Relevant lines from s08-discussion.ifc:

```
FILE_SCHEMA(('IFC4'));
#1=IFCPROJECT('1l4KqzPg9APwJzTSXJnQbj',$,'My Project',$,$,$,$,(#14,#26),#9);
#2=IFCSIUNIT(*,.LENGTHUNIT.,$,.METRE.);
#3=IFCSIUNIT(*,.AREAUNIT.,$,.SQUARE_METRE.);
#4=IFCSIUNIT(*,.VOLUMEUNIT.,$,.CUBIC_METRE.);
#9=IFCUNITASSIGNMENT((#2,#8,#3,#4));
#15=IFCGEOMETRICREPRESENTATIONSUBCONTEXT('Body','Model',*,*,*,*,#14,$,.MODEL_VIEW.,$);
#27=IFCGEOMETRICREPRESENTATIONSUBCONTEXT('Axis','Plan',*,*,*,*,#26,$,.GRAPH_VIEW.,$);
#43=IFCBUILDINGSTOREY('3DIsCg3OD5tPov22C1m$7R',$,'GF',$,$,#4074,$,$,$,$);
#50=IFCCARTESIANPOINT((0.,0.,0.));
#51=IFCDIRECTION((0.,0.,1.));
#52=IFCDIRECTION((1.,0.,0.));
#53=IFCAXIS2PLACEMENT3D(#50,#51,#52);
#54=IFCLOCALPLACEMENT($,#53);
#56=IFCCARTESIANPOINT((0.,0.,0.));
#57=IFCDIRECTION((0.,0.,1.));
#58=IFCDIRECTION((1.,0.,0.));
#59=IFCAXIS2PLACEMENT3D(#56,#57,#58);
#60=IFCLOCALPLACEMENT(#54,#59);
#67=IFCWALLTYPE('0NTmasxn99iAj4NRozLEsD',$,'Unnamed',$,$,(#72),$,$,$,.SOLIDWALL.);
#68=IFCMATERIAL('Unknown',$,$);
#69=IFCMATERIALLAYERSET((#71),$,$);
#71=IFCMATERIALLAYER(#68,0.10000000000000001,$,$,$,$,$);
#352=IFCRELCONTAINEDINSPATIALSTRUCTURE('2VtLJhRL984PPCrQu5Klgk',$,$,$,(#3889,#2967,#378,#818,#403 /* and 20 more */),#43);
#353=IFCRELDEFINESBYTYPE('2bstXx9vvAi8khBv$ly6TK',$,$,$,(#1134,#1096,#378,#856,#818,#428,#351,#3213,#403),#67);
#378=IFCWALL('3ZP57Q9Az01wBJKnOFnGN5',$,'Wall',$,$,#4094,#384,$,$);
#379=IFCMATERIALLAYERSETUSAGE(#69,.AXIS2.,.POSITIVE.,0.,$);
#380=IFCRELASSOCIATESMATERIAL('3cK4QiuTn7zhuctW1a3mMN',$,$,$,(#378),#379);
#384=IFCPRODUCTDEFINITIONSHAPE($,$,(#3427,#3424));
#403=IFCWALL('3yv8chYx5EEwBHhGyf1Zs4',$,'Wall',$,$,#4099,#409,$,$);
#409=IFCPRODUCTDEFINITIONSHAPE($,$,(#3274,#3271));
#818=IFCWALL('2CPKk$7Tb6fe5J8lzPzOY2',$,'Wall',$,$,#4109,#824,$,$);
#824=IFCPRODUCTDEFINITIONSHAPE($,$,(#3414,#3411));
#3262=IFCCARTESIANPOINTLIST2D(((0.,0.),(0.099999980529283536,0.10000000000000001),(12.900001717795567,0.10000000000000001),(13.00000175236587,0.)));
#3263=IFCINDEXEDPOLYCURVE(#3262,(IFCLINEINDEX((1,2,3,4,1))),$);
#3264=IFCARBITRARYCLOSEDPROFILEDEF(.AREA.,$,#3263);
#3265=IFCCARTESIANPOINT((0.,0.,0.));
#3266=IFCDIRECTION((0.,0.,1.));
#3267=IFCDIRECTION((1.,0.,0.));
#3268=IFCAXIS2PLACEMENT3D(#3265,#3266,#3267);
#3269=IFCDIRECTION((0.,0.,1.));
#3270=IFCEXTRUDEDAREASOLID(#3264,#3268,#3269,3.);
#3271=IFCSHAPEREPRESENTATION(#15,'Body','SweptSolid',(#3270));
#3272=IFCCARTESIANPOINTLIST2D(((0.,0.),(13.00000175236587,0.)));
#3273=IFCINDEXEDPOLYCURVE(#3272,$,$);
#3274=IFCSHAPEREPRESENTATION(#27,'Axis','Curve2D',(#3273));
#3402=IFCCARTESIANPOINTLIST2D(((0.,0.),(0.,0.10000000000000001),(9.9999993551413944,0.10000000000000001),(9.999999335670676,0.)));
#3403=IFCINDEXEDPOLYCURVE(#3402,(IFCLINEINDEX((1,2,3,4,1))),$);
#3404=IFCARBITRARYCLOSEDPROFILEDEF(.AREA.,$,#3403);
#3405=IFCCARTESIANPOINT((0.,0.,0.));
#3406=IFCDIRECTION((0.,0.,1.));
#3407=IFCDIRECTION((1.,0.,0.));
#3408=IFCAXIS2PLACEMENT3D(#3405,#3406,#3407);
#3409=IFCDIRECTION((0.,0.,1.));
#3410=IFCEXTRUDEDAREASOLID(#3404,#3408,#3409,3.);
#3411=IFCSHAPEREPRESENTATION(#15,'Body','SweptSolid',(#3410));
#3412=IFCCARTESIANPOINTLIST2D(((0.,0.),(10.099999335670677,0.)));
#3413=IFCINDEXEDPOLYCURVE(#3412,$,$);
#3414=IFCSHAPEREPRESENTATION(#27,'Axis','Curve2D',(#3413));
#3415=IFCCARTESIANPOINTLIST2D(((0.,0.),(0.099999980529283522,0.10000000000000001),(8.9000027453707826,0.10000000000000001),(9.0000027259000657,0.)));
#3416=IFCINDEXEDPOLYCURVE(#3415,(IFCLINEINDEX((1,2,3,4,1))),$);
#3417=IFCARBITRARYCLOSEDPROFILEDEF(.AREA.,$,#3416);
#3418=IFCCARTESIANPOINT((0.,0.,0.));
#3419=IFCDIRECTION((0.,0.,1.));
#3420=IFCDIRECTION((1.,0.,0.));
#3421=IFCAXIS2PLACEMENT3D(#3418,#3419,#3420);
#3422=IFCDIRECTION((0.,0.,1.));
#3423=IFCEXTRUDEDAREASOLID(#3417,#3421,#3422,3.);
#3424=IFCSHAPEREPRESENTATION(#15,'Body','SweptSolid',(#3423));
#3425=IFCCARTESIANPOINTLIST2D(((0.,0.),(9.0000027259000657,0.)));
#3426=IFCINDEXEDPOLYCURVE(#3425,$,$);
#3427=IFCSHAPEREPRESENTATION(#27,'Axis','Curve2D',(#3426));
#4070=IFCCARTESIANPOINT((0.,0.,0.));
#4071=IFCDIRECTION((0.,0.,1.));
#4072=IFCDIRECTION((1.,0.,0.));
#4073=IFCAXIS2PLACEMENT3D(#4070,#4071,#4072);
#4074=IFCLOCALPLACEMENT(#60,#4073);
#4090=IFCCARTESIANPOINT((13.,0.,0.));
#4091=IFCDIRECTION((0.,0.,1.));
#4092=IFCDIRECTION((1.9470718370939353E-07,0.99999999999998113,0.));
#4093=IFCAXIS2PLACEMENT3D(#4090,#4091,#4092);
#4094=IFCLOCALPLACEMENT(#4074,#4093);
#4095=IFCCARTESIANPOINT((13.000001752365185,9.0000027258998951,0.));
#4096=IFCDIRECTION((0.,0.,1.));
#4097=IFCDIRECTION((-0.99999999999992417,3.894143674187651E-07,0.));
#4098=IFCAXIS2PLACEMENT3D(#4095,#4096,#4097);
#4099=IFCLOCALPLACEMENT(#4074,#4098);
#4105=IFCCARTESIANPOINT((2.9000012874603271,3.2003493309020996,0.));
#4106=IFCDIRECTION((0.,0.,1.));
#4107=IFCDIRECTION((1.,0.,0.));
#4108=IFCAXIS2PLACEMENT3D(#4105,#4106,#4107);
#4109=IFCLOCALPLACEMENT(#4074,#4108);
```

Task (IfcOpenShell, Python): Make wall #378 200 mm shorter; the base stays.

```python
import ifcopenshell
import ifcopenshell.geom
import ifcopenshell.util.representation
import ifcopenshell.util.shape

model = ifcopenshell.open("s08-discussion.ifc")
settings = ifcopenshell.geom.settings()


def volume(element):
    """Net volume in cubic metres, openings subtracted."""
    shape = ifcopenshell.geom.create_shape(settings, element)
    return ifcopenshell.util.shape.get_volume(shape.geometry)


wall = model.by_guid("3ZP57Q9Az01wBJKnOFnGN5")
before = volume(wall)

body = ifcopenshell.util.representation.get_representation(wall, "Model", "Body")
solid = body.Items[0]
old_height = solid.Depth
solid.Depth -= 0.2
after = volume(wall)

print(f"height {old_height:g} -> {solid.Depth:g}, volume {before:.3f} -> {after:.3f} m3")

model.write("s08-discussion_edited.ifc")
```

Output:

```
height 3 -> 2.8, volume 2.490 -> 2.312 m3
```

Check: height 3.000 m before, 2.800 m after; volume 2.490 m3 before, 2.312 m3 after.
